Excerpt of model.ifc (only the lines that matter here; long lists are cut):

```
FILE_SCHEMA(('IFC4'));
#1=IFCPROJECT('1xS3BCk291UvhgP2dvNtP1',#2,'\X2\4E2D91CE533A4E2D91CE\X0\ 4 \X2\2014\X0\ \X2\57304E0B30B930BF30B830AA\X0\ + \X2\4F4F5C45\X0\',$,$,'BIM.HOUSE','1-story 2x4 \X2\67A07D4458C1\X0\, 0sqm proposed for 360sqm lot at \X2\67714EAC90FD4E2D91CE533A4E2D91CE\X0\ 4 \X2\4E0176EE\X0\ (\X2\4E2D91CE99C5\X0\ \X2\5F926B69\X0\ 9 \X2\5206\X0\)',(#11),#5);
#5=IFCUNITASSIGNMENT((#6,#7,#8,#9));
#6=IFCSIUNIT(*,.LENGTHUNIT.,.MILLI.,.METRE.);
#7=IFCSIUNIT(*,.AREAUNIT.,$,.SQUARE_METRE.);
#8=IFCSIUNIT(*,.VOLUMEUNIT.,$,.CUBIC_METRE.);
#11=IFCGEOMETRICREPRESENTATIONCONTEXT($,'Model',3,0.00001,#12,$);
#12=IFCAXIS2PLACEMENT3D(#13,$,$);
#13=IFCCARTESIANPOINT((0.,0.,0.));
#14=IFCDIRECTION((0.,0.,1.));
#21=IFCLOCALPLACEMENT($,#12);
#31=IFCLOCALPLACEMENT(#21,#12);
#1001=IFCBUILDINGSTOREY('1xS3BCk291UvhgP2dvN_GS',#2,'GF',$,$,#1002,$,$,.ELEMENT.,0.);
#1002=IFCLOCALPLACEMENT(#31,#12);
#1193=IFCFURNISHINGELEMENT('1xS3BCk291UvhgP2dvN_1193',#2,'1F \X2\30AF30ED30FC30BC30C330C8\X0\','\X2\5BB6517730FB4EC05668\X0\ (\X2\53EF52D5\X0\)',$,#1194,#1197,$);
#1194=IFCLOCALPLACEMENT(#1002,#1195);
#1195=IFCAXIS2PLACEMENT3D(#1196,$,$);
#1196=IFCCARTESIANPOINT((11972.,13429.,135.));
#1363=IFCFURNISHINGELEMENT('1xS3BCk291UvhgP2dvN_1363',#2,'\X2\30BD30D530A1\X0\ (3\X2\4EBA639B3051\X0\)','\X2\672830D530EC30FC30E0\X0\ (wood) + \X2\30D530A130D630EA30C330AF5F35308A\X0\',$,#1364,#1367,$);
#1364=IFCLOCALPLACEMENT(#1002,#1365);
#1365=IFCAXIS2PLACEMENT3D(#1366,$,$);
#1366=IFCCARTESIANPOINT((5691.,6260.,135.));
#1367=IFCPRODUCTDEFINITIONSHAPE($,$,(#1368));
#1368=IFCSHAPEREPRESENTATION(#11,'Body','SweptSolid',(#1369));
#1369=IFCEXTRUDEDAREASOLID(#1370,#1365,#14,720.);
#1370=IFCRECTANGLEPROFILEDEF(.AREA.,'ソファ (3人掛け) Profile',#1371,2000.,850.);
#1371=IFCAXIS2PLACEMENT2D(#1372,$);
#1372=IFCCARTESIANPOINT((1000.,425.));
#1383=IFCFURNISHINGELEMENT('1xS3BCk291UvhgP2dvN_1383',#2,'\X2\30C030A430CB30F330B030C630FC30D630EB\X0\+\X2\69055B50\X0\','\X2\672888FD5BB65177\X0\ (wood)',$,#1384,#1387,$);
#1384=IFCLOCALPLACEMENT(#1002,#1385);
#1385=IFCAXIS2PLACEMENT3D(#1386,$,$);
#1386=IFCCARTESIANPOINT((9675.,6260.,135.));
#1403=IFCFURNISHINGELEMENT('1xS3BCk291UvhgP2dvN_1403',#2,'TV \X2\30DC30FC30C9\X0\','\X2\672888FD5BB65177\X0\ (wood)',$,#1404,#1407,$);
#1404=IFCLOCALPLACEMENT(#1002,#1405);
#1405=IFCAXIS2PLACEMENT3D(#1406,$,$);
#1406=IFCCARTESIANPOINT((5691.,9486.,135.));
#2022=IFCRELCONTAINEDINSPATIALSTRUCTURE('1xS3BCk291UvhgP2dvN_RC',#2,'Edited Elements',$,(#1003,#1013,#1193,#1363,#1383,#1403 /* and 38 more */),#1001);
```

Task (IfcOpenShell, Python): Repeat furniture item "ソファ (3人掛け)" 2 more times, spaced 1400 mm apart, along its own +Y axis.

```python
import ifcopenshell
import ifcopenshell.api.geometry
import ifcopenshell.api.root
import ifcopenshell.util.element
import ifcopenshell.util.placement
import ifcopenshell.util.unit

model = ifcopenshell.open("model.ifc")
unit_scale = ifcopenshell.util.unit.calculate_unit_scale(model)


def reuse_history(source, copy):
    """copy_class also copies each property set's owner history, people and application; keep the originals."""
    for rel in copy.IsDefinedBy:
        if rel.is_a("IfcRelDefinesByProperties") and (history := rel.RelatingPropertyDefinition.OwnerHistory):
            rel.RelatingPropertyDefinition.OwnerHistory = source.OwnerHistory
            ifcopenshell.util.element.remove_deep2(model, history)


source = model.by_id(1363)
base = ifcopenshell.util.placement.get_local_placement(source.ObjectPlacement)
step = base[:3, 1] * 1.4 / unit_scale

for i in range(1, 3):
    copy = ifcopenshell.api.root.copy_class(model, product=source)
    copy.Representation = ifcopenshell.util.element.copy_deep(
        model, source.Representation, exclude=["IfcGeometricRepresentationContext", "IfcRepresentationMap"]
    )
    reuse_history(source, copy)
    matrix = base.copy()
    matrix[:3, 3] += i * step
    print("added at", matrix[:3, 3].round(3) + 0.0)
    ifcopenshell.api.geometry.edit_object_placement(model, product=copy, matrix=matrix, is_si=False)

model.write("model_updated.ifc")
```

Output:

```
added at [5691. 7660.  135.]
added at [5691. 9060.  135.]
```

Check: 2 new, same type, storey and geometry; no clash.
